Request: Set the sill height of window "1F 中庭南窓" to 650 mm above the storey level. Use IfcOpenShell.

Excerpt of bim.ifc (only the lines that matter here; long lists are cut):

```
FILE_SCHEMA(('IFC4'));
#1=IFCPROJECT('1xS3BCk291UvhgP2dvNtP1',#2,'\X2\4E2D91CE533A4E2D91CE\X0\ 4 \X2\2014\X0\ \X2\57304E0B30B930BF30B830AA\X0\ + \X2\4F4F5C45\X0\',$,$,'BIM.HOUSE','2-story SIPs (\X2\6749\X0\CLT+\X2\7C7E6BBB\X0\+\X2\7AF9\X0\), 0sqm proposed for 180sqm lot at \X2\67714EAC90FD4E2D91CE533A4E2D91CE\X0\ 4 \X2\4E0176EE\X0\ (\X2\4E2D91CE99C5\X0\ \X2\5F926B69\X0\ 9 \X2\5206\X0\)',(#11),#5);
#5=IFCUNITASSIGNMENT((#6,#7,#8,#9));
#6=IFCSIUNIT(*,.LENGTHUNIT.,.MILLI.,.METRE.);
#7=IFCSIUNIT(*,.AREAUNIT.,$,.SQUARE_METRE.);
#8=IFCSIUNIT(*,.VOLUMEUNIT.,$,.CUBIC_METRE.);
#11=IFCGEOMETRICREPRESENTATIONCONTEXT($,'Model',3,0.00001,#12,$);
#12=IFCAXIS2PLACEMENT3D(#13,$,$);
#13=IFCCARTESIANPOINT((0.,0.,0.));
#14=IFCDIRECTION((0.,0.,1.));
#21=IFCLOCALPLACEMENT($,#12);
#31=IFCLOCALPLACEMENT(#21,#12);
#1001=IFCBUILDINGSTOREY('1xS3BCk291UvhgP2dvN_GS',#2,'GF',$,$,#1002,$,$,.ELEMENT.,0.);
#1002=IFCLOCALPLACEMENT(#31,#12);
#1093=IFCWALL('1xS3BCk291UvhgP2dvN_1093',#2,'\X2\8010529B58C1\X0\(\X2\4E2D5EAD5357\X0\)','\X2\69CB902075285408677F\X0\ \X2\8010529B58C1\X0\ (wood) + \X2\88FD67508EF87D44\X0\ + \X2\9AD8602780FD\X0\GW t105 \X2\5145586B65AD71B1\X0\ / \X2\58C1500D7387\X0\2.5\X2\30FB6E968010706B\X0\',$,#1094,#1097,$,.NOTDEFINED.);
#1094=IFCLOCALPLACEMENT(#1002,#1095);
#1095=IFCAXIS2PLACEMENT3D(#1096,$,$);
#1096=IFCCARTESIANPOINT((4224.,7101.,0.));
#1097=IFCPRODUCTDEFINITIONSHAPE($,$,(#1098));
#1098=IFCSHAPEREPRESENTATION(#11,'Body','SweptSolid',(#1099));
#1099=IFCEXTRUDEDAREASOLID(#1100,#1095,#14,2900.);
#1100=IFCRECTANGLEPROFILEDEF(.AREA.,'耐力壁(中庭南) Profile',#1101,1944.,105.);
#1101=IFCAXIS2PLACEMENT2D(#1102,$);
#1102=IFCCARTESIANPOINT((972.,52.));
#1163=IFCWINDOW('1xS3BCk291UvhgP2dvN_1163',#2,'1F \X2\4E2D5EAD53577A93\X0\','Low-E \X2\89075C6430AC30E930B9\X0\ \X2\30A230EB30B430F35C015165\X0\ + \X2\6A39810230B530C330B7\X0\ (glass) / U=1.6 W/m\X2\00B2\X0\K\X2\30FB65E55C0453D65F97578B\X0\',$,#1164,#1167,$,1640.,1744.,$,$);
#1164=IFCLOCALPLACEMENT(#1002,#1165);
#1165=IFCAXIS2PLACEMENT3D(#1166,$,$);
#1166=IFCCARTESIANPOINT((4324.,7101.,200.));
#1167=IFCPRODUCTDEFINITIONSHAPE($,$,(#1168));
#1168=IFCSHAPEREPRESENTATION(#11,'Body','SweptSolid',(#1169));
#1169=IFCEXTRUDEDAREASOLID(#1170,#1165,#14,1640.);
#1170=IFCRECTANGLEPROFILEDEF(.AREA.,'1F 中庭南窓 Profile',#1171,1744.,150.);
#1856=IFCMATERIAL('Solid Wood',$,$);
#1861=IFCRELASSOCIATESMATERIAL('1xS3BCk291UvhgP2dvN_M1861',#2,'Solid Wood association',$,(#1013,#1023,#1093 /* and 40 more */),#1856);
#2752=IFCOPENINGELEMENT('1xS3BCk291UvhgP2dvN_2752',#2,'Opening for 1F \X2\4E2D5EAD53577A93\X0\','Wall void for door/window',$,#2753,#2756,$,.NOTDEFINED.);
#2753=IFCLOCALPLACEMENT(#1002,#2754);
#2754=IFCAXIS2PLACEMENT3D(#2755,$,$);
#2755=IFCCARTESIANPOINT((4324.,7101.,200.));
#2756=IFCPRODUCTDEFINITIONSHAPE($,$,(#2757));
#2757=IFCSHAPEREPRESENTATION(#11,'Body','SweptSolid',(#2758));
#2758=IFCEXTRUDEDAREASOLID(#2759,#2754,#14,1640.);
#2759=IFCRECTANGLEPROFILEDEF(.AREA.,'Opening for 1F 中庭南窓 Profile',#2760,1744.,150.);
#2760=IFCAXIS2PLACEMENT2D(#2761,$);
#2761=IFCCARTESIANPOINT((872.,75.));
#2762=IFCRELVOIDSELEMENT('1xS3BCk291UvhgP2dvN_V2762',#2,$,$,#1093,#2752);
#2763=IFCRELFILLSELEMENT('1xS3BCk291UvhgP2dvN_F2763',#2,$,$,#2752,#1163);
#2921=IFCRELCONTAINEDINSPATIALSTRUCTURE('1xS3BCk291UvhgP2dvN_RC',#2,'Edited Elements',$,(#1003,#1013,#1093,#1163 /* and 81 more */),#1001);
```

```python
import numpy as np
import ifcopenshell
import ifcopenshell.api.geometry
import ifcopenshell.geom
import ifcopenshell.util.element
import ifcopenshell.util.placement
import ifcopenshell.util.shape
import ifcopenshell.util.unit

model = ifcopenshell.open("bim.ifc")
unit_scale = ifcopenshell.util.unit.calculate_unit_scale(model)

window = model.by_guid("1xS3BCk291UvhgP2dvN_1163")
opening = window.FillsVoids[0].RelatingOpeningElement
storey = ifcopenshell.util.element.get_container(window, ifc_class="IfcBuildingStorey")
level = ifcopenshell.util.placement.get_local_placement(storey.ObjectPlacement)[2, 3]

# The opening's origin need not be at the sill, so measure its lowest point.
shape = ifcopenshell.geom.create_shape(ifcopenshell.geom.settings(), opening)
bottom = ifcopenshell.util.shape.get_shape_bottom_elevation(shape, shape.geometry) / unit_scale
dz = level + 0.65 / unit_scale - bottom

shift = np.array([0.0, 0.0, dz])
# The window is not placed relative to its opening, so move both.
for product in (opening, window):
    matrix = ifcopenshell.util.placement.get_local_placement(product.ObjectPlacement)
    matrix[:3, 3] += shift
    ifcopenshell.api.geometry.edit_object_placement(model, product=product, matrix=matrix, is_si=False)

print(f"moved by {dz * unit_scale:+.3f} m")

model.write("bim_edited.ifc")
```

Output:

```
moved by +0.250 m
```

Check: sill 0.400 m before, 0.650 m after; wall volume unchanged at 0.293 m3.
